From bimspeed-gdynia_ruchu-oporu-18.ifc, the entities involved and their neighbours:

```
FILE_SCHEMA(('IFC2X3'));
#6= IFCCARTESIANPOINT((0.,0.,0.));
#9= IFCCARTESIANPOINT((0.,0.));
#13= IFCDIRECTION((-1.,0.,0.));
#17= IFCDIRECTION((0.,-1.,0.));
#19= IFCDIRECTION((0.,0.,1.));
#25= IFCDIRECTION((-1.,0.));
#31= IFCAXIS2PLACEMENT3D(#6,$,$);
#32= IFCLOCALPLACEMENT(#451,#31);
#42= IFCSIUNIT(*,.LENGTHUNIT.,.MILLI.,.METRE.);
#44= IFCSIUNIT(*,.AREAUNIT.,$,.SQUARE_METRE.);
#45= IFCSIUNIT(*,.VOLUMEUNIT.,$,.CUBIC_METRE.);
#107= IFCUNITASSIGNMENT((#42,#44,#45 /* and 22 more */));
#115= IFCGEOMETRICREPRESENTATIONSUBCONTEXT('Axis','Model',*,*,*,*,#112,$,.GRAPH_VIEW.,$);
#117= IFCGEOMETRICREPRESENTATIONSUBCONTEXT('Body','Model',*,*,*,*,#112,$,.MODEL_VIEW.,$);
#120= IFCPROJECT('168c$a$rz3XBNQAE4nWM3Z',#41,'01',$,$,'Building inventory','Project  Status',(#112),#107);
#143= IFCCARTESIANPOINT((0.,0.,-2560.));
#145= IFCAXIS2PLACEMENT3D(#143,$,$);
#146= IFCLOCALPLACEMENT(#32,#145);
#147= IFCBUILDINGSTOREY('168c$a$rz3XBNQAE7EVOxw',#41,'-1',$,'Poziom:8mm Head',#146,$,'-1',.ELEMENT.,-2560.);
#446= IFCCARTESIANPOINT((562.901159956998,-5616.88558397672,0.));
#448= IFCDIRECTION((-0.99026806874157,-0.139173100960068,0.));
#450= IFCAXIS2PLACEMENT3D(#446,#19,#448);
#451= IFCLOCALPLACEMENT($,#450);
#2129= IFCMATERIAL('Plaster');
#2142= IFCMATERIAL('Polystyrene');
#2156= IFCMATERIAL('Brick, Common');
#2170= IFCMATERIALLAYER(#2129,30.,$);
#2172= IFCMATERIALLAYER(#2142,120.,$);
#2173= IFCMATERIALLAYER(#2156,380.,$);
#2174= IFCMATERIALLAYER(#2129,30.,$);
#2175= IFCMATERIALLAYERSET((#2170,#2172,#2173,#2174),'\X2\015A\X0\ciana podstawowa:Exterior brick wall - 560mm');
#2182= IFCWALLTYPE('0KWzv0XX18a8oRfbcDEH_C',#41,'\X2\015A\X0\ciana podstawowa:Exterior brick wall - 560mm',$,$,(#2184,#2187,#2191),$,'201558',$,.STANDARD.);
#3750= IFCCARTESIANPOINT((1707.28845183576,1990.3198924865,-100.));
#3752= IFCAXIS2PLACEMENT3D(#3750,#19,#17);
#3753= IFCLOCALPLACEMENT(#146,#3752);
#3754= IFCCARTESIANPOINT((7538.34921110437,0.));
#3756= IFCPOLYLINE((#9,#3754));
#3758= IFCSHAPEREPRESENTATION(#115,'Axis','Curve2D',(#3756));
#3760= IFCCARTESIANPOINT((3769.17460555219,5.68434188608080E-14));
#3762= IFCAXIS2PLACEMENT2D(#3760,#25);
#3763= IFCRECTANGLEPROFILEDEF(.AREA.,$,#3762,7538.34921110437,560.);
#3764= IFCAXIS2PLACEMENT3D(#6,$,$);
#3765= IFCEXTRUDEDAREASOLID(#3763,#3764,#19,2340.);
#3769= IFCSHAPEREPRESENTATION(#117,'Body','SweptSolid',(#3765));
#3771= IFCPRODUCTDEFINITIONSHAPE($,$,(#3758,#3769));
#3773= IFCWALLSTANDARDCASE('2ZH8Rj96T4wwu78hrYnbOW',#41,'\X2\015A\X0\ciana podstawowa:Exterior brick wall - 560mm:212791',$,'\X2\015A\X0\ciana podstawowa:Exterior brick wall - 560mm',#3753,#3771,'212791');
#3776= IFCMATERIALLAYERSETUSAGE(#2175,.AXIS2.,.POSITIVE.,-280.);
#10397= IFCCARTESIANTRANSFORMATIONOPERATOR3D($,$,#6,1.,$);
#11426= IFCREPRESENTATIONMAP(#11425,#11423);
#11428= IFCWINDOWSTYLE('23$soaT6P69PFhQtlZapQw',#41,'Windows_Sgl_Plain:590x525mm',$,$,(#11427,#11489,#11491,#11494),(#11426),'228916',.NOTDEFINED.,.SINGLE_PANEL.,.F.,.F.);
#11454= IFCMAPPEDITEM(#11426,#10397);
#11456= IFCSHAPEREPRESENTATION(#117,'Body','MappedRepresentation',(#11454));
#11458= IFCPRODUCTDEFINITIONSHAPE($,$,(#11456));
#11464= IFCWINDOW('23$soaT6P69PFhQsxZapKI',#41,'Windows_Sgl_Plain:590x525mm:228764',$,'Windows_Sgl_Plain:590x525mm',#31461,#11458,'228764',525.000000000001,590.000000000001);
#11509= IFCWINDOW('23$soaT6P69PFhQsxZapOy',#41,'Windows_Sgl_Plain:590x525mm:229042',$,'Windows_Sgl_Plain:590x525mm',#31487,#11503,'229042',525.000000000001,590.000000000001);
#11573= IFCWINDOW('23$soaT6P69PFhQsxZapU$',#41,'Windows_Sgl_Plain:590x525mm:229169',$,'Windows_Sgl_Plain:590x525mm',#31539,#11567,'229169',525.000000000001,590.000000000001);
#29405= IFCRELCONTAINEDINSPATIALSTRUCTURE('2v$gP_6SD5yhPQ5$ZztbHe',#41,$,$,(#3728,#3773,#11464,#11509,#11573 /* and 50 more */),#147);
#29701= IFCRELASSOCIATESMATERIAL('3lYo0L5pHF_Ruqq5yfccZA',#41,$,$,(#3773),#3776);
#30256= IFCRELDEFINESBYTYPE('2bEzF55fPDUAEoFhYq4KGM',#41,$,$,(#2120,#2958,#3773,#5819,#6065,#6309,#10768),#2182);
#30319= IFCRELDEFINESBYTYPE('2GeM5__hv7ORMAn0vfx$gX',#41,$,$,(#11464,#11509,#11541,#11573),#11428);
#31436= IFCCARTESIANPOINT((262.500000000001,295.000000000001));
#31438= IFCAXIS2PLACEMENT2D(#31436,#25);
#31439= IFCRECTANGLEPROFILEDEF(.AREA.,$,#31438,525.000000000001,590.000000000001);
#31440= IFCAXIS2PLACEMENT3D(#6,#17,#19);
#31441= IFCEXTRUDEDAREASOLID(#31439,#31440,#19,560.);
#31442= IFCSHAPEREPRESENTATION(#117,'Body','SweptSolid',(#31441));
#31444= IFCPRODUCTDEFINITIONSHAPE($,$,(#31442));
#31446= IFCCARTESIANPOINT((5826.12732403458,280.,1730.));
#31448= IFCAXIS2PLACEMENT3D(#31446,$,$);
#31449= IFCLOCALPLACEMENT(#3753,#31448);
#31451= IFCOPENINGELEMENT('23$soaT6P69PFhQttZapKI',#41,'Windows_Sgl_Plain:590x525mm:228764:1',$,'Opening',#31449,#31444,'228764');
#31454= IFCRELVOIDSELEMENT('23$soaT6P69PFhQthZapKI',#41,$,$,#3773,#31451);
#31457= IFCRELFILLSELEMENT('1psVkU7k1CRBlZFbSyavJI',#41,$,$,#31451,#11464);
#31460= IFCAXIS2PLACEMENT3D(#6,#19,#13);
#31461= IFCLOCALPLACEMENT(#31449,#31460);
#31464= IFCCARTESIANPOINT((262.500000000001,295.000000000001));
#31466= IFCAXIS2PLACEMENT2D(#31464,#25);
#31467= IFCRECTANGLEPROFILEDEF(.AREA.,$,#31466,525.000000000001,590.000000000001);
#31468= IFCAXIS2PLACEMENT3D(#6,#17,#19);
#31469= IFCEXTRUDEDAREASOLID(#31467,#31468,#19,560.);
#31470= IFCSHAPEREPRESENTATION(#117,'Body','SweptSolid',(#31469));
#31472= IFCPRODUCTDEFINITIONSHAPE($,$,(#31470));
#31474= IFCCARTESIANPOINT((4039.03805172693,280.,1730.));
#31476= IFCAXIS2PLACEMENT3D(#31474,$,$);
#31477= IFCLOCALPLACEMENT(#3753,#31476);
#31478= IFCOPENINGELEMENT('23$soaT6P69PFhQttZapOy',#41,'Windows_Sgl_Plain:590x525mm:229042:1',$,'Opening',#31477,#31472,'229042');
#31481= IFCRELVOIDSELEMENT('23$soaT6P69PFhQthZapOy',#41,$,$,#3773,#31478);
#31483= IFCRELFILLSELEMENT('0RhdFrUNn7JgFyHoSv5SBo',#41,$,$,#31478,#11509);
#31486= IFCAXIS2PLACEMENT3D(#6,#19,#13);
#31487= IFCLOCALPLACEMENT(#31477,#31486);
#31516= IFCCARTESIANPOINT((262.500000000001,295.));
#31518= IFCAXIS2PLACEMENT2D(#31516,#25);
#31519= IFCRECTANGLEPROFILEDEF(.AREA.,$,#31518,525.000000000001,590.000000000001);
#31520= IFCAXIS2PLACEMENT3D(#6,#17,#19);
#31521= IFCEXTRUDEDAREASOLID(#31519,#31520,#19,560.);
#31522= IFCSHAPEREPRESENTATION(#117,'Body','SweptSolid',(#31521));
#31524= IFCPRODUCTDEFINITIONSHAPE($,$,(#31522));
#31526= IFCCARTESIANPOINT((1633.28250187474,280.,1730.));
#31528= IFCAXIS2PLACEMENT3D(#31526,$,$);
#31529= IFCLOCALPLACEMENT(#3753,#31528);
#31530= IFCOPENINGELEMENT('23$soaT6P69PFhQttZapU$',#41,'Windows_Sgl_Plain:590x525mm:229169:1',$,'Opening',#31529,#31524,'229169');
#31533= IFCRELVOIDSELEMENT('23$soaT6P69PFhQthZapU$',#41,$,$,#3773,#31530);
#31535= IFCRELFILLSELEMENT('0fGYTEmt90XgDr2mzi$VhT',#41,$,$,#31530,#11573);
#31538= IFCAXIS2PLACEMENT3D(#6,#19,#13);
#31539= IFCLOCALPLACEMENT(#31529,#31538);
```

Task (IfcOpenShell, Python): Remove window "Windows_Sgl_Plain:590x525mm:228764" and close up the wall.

```python
import ifcopenshell
import ifcopenshell.api.feature
import ifcopenshell.api.root
import ifcopenshell.geom
import ifcopenshell.util.shape

model = ifcopenshell.open("bimspeed-gdynia_ruchu-oporu-18.ifc")
settings = ifcopenshell.geom.settings()


def volume(element):
    """Net volume in cubic metres, openings subtracted."""
    shape = ifcopenshell.geom.create_shape(settings, element)
    return ifcopenshell.util.shape.get_volume(shape.geometry)


window = model.by_guid("23$soaT6P69PFhQsxZapKI")
opening = window.FillsVoids[0].RelatingOpeningElement
wall = opening.VoidsElements[0].RelatingBuildingElement
before = volume(wall)

ifcopenshell.api.root.remove_product(model, product=window)
ifcopenshell.api.feature.remove_feature(model, feature=opening)

after = volume(wall)

print(f"wall volume {before:.3f} -> {after:.3f} m3")

model.write("bimspeed-gdynia_ruchu-oporu-18_edited.ifc")
```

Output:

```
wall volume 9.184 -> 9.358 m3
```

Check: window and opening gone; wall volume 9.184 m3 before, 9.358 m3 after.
